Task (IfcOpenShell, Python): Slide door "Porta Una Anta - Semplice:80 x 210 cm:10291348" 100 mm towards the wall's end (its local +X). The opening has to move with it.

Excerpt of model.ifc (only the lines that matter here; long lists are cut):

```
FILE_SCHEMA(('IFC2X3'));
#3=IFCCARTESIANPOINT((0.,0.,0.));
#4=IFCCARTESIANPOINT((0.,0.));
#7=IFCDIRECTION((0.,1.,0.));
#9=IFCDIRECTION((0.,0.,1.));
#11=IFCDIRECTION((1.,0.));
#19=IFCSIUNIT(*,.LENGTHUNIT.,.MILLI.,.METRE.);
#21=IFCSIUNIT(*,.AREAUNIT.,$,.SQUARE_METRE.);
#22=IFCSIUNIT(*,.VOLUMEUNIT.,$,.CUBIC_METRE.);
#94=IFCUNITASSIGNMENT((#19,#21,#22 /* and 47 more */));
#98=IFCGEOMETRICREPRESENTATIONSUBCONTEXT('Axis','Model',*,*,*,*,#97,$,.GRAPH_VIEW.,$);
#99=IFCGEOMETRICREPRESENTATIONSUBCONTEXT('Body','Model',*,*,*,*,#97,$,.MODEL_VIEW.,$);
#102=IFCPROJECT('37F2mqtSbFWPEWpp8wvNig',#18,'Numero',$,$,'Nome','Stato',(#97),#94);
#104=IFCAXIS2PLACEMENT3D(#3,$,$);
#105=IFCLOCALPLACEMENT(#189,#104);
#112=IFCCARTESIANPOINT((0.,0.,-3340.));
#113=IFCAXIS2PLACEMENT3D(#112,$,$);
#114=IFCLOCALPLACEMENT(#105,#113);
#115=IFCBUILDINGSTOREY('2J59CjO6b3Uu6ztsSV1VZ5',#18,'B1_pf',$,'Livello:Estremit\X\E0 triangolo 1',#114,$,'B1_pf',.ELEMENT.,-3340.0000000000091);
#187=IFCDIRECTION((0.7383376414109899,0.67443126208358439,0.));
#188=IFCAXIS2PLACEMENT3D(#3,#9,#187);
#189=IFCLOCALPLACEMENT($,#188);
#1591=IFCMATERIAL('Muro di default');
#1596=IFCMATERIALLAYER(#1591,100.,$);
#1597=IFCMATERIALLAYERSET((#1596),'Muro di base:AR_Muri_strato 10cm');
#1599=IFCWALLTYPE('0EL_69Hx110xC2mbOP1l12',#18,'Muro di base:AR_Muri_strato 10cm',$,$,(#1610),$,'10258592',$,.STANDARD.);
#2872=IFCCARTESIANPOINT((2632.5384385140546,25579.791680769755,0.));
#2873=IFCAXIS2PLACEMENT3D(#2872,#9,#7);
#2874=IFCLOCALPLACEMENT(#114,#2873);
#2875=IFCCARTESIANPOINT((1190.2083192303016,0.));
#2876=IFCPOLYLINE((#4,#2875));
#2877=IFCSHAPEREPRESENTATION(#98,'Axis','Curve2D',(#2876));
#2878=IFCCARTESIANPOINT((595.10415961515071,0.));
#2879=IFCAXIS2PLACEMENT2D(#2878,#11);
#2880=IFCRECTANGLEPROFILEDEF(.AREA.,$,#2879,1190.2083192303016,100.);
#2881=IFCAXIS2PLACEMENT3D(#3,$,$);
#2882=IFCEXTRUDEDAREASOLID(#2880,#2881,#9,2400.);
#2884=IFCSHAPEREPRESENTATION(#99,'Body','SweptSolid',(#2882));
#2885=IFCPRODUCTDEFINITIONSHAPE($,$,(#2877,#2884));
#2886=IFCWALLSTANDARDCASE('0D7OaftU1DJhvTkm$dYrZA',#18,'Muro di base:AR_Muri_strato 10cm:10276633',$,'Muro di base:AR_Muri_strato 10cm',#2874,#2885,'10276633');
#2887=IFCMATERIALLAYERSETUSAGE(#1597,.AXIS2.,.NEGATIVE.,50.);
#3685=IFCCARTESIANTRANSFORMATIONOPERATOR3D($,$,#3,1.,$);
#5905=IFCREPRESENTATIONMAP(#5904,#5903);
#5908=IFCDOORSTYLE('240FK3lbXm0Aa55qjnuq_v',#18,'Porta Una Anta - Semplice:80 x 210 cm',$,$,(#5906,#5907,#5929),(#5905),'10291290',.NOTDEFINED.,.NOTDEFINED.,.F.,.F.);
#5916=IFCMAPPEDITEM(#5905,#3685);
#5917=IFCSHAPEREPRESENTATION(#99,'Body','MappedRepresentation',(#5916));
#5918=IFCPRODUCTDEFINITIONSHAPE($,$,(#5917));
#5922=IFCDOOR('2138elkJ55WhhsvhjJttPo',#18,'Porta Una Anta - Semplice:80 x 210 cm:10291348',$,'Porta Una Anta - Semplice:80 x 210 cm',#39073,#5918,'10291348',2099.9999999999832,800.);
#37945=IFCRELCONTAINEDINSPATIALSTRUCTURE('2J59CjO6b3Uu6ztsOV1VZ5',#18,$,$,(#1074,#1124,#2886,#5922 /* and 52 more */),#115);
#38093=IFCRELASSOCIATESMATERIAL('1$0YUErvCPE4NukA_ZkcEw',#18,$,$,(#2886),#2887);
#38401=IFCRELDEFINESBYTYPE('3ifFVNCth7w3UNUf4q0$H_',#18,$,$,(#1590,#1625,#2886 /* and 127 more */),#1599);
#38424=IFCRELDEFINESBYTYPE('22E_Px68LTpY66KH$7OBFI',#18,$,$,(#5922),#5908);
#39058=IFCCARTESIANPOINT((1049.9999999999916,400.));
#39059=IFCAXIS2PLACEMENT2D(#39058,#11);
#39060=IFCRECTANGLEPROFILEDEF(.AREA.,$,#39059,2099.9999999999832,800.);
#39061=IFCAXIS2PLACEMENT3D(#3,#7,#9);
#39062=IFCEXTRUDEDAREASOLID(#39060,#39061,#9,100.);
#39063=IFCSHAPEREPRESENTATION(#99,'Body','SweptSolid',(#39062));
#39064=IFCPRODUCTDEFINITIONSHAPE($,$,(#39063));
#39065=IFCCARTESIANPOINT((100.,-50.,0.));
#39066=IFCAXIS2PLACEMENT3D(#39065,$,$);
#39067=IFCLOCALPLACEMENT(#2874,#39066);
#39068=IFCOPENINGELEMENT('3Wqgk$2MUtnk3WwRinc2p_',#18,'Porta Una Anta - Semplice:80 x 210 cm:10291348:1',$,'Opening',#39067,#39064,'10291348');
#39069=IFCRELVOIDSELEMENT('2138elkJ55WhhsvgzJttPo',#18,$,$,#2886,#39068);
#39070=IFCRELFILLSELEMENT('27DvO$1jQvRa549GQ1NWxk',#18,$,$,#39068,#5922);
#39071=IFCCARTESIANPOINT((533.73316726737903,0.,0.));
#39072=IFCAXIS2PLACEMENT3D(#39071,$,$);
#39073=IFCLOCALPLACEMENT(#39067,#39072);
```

```python
import ifcopenshell
import ifcopenshell.api.geometry
import ifcopenshell.util.placement
import ifcopenshell.util.unit

model = ifcopenshell.open("model.ifc")
unit_scale = ifcopenshell.util.unit.calculate_unit_scale(model)

door = model.by_guid("2138elkJ55WhhsvhjJttPo")
opening = door.FillsVoids[0].RelatingOpeningElement
wall = opening.VoidsElements[0].RelatingBuildingElement

wall_matrix = ifcopenshell.util.placement.get_local_placement(wall.ObjectPlacement)
shift = wall_matrix[:3, 0] * 0.1 / unit_scale
before = ifcopenshell.util.placement.get_local_placement(door.ObjectPlacement)[:3, 3].copy()

# The door is placed relative to its opening, so it follows when the opening moves.
matrix = ifcopenshell.util.placement.get_local_placement(opening.ObjectPlacement)
matrix[:3, 3] += shift
ifcopenshell.api.geometry.edit_object_placement(
    model, product=opening, matrix=matrix, is_si=False, should_transform_children=True
)

after = ifcopenshell.util.placement.get_local_placement(door.ObjectPlacement)[:3, 3]
print("door moved by", (after - before).round(3) + 0.0)

model.write("model_updated.ifc")
```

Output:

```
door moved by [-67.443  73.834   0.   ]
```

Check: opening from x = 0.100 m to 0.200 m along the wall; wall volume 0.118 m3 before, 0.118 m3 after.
